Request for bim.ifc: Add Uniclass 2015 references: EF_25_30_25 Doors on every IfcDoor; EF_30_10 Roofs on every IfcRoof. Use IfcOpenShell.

First a look at what the model holds.

```python
import ifcopenshell

model = ifcopenshell.open("bim.ifc")
print(model.schema)
print("classifications:", [c.Name for c in model.by_type("IfcClassification")])
for ifc_class in ("IfcDoor", "IfcRoof", "IfcStair", "IfcWall", "IfcWindow"):
    print(ifc_class, len(model.by_type(ifc_class)))
```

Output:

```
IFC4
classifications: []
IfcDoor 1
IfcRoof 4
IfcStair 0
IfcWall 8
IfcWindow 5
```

```python
import ifcopenshell
import ifcopenshell.api.classification

model = ifcopenshell.open("bim.ifc")

system = ifcopenshell.api.classification.add_classification(model, classification="Uniclass 2015")

codes = {
    "IfcDoor": ("EF_25_30_25", "Doors"),
    "IfcRoof": ("EF_30_10", "Roofs"),
}
for ifc_class, (code, name) in codes.items():
    products = model.by_type(ifc_class)
    ifcopenshell.api.classification.add_reference(
        model, products=products, classification=system, identification=code, name=name
    )
    print(code, len(products))

model.write("bim-out.ifc")
```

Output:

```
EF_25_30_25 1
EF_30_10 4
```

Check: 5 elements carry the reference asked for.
